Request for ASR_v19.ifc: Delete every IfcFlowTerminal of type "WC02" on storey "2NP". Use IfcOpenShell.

First a look at what the model holds.

```python
import ifcopenshell
import ifcopenshell.util.element

model = ifcopenshell.open("ASR_v19.ifc")
print(model.schema)
storey = next(s for s in model.by_type("IfcBuildingStorey") if s.Name == "2NP")
terminals = [e for e in ifcopenshell.util.element.get_decomposition(storey) if e.is_a("IfcFlowTerminal")]
seen = {}
for e in terminals:
    element_type = ifcopenshell.util.element.get_type(e)
    name = element_type.Name if element_type not in (None, e) else None
    seen[name] = seen.get(name, 0) + 1
for name, count in sorted(seen.items(), key=str):
    print(count, "x", name)
```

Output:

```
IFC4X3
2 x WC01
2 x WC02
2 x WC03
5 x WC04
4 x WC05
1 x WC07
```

```python
import ifcopenshell
import ifcopenshell.api.root
import ifcopenshell.util.element

model = ifcopenshell.open("ASR_v19.ifc")

storey = next(s for s in model.by_type("IfcBuildingStorey") if s.Name == "2NP")
terminals = [e for e in ifcopenshell.util.element.get_decomposition(storey) if e.is_a("IfcFlowTerminal")]
targets = [e for e in terminals if (t := ifcopenshell.util.element.get_type(e)) not in (None, e) and t.Name == "WC02"]

for e in targets:
    ifcopenshell.api.root.remove_product(model, product=e)
print(len(targets), "removed")

model.write("ASR_v19_v2.ifc")
```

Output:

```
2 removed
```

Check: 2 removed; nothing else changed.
